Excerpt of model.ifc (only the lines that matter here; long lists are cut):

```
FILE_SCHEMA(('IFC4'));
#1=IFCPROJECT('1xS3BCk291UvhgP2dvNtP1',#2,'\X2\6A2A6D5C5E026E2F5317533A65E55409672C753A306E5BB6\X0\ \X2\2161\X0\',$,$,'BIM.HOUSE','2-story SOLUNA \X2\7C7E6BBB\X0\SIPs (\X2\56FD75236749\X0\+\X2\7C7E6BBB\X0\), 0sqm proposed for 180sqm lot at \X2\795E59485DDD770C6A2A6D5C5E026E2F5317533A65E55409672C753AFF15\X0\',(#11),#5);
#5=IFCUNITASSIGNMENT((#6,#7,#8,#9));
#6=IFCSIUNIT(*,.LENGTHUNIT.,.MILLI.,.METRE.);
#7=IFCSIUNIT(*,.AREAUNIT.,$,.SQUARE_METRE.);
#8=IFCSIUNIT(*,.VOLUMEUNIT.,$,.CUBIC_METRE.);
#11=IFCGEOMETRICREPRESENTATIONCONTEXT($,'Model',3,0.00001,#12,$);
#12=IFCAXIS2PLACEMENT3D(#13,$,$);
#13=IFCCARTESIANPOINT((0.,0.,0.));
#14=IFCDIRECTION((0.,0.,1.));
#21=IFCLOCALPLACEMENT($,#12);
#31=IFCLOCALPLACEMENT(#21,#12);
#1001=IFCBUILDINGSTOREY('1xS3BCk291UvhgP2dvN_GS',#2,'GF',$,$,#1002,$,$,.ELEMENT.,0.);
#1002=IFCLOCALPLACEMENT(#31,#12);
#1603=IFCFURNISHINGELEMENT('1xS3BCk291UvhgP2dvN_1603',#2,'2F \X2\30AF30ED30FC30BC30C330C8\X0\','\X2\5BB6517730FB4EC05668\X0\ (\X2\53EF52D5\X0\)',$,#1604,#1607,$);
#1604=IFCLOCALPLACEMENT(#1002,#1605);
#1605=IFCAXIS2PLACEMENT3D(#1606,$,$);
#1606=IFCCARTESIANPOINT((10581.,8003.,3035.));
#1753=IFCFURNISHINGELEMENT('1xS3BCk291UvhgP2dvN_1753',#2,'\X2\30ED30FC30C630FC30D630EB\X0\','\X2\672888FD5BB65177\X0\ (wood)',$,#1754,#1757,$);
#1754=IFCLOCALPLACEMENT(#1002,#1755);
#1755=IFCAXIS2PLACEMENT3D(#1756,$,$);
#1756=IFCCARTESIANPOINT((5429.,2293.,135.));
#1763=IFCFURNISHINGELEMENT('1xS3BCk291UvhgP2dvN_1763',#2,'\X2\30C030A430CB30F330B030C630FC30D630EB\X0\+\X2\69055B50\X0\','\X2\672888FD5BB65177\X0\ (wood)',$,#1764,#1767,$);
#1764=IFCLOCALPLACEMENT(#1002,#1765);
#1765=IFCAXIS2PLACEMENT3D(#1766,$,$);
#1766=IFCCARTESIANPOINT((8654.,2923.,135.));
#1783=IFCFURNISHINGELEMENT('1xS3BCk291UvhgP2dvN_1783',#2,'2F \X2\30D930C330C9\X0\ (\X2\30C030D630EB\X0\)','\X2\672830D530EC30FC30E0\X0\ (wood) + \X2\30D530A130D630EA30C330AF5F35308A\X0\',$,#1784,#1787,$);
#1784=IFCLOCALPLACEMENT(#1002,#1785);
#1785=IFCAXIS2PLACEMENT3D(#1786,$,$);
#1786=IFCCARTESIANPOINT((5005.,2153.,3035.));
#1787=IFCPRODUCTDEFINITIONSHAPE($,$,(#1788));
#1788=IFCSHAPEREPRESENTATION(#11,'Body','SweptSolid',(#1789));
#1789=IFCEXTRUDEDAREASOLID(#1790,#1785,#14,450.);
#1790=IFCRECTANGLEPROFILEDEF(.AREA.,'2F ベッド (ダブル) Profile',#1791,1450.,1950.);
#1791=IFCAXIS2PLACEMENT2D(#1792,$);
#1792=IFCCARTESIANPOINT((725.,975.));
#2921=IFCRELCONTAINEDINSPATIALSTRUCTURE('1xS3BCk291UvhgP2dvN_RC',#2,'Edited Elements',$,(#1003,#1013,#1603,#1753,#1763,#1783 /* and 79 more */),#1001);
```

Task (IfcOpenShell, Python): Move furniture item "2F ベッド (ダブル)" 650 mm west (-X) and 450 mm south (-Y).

```python
import ifcopenshell
import ifcopenshell.api.geometry
import ifcopenshell.util.placement
import ifcopenshell.util.unit

model = ifcopenshell.open("model.ifc")
unit_scale = ifcopenshell.util.unit.calculate_unit_scale(model)

item = model.by_guid("1xS3BCk291UvhgP2dvN_1783")
matrix = ifcopenshell.util.placement.get_local_placement(item.ObjectPlacement)
matrix[0, 3] -= 0.65 / unit_scale
matrix[1, 3] -= 0.45 / unit_scale
ifcopenshell.api.geometry.edit_object_placement(model, product=item, matrix=matrix, is_si=False)

print(ifcopenshell.util.placement.get_local_placement(item.ObjectPlacement).round(3) + 0.0)

model.write("model_edited.ifc")
```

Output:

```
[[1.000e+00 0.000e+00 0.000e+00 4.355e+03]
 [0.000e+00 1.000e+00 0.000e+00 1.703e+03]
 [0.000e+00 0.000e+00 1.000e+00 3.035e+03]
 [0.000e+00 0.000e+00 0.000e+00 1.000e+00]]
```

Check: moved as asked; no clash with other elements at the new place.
